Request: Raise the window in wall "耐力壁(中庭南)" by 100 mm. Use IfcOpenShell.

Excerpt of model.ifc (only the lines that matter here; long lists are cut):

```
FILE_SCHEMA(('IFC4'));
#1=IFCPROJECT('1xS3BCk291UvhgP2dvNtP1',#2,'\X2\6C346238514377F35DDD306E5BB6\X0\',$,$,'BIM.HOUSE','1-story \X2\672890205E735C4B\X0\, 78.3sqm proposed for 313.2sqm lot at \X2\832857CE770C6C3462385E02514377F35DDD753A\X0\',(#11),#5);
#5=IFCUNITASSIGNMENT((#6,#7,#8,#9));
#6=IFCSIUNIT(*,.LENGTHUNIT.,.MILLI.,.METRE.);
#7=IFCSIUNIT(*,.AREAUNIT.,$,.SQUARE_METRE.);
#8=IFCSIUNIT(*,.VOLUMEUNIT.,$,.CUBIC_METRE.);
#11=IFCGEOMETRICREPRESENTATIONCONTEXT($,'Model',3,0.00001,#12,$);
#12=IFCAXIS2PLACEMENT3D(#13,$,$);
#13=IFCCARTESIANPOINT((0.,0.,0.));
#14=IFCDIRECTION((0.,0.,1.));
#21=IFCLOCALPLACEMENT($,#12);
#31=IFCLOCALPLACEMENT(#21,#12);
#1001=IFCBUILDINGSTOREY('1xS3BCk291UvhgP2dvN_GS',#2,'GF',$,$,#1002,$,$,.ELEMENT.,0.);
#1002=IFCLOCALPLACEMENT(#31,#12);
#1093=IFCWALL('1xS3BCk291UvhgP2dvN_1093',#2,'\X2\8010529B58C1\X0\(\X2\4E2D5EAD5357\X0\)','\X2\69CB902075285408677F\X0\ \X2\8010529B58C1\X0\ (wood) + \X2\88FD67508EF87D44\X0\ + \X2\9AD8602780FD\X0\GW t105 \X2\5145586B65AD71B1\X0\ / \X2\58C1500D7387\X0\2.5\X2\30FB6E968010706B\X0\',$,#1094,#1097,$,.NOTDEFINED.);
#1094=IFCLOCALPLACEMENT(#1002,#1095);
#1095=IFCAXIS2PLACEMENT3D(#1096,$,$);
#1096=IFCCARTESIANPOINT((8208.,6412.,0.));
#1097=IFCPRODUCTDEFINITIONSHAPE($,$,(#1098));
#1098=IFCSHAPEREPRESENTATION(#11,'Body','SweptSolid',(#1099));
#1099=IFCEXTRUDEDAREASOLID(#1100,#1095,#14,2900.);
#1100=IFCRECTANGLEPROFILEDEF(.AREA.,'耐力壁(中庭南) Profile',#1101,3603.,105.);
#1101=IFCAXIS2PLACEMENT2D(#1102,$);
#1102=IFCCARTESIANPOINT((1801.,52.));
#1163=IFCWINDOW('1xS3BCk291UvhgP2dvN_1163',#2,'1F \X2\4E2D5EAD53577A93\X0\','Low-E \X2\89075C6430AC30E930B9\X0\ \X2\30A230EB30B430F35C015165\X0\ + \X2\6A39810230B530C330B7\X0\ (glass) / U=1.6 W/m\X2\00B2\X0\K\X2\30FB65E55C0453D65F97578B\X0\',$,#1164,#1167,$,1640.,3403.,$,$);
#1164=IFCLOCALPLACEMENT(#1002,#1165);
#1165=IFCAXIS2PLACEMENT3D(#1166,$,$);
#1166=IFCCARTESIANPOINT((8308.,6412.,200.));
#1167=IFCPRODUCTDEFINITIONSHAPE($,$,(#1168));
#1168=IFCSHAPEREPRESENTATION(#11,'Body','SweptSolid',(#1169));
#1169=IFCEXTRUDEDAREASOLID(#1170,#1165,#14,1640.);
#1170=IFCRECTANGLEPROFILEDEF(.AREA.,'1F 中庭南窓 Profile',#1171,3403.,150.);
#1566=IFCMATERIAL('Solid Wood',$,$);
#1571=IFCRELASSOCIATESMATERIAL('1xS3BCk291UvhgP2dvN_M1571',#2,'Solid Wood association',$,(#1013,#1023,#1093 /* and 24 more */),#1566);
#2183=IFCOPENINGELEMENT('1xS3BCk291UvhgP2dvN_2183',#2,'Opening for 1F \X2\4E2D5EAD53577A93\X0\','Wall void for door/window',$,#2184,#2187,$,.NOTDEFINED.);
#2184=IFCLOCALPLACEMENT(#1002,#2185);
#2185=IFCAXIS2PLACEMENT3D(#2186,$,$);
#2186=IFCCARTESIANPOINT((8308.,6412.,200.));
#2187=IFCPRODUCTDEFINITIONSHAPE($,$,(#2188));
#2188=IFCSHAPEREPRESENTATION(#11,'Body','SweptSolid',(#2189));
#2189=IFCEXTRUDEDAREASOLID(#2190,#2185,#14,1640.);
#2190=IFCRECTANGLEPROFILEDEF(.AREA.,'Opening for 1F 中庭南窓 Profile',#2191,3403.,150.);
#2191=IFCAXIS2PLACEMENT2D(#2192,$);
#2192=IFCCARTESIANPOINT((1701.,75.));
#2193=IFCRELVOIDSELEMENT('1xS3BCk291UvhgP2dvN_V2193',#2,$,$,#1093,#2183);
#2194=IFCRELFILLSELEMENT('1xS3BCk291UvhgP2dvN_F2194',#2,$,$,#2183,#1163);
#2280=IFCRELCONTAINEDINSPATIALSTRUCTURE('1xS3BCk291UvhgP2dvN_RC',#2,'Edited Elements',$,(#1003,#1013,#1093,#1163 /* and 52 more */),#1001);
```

```python
import numpy as np
import ifcopenshell
import ifcopenshell.api.geometry
import ifcopenshell.util.placement
import ifcopenshell.util.unit

model = ifcopenshell.open("model.ifc")
unit_scale = ifcopenshell.util.unit.calculate_unit_scale(model)

window = model.by_id(1163)
opening = window.FillsVoids[0].RelatingOpeningElement
dz = 0.1 / unit_scale

shift = np.array([0.0, 0.0, dz])
# The window is not placed relative to its opening, so move both.
for product in (opening, window):
    matrix = ifcopenshell.util.placement.get_local_placement(product.ObjectPlacement)
    matrix[:3, 3] += shift
    ifcopenshell.api.geometry.edit_object_placement(model, product=product, matrix=matrix, is_si=False)

print(f"moved by {dz * unit_scale:+.3f} m")

model.write("model-out.ifc")
```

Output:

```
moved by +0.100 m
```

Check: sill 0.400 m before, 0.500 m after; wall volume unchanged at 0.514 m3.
